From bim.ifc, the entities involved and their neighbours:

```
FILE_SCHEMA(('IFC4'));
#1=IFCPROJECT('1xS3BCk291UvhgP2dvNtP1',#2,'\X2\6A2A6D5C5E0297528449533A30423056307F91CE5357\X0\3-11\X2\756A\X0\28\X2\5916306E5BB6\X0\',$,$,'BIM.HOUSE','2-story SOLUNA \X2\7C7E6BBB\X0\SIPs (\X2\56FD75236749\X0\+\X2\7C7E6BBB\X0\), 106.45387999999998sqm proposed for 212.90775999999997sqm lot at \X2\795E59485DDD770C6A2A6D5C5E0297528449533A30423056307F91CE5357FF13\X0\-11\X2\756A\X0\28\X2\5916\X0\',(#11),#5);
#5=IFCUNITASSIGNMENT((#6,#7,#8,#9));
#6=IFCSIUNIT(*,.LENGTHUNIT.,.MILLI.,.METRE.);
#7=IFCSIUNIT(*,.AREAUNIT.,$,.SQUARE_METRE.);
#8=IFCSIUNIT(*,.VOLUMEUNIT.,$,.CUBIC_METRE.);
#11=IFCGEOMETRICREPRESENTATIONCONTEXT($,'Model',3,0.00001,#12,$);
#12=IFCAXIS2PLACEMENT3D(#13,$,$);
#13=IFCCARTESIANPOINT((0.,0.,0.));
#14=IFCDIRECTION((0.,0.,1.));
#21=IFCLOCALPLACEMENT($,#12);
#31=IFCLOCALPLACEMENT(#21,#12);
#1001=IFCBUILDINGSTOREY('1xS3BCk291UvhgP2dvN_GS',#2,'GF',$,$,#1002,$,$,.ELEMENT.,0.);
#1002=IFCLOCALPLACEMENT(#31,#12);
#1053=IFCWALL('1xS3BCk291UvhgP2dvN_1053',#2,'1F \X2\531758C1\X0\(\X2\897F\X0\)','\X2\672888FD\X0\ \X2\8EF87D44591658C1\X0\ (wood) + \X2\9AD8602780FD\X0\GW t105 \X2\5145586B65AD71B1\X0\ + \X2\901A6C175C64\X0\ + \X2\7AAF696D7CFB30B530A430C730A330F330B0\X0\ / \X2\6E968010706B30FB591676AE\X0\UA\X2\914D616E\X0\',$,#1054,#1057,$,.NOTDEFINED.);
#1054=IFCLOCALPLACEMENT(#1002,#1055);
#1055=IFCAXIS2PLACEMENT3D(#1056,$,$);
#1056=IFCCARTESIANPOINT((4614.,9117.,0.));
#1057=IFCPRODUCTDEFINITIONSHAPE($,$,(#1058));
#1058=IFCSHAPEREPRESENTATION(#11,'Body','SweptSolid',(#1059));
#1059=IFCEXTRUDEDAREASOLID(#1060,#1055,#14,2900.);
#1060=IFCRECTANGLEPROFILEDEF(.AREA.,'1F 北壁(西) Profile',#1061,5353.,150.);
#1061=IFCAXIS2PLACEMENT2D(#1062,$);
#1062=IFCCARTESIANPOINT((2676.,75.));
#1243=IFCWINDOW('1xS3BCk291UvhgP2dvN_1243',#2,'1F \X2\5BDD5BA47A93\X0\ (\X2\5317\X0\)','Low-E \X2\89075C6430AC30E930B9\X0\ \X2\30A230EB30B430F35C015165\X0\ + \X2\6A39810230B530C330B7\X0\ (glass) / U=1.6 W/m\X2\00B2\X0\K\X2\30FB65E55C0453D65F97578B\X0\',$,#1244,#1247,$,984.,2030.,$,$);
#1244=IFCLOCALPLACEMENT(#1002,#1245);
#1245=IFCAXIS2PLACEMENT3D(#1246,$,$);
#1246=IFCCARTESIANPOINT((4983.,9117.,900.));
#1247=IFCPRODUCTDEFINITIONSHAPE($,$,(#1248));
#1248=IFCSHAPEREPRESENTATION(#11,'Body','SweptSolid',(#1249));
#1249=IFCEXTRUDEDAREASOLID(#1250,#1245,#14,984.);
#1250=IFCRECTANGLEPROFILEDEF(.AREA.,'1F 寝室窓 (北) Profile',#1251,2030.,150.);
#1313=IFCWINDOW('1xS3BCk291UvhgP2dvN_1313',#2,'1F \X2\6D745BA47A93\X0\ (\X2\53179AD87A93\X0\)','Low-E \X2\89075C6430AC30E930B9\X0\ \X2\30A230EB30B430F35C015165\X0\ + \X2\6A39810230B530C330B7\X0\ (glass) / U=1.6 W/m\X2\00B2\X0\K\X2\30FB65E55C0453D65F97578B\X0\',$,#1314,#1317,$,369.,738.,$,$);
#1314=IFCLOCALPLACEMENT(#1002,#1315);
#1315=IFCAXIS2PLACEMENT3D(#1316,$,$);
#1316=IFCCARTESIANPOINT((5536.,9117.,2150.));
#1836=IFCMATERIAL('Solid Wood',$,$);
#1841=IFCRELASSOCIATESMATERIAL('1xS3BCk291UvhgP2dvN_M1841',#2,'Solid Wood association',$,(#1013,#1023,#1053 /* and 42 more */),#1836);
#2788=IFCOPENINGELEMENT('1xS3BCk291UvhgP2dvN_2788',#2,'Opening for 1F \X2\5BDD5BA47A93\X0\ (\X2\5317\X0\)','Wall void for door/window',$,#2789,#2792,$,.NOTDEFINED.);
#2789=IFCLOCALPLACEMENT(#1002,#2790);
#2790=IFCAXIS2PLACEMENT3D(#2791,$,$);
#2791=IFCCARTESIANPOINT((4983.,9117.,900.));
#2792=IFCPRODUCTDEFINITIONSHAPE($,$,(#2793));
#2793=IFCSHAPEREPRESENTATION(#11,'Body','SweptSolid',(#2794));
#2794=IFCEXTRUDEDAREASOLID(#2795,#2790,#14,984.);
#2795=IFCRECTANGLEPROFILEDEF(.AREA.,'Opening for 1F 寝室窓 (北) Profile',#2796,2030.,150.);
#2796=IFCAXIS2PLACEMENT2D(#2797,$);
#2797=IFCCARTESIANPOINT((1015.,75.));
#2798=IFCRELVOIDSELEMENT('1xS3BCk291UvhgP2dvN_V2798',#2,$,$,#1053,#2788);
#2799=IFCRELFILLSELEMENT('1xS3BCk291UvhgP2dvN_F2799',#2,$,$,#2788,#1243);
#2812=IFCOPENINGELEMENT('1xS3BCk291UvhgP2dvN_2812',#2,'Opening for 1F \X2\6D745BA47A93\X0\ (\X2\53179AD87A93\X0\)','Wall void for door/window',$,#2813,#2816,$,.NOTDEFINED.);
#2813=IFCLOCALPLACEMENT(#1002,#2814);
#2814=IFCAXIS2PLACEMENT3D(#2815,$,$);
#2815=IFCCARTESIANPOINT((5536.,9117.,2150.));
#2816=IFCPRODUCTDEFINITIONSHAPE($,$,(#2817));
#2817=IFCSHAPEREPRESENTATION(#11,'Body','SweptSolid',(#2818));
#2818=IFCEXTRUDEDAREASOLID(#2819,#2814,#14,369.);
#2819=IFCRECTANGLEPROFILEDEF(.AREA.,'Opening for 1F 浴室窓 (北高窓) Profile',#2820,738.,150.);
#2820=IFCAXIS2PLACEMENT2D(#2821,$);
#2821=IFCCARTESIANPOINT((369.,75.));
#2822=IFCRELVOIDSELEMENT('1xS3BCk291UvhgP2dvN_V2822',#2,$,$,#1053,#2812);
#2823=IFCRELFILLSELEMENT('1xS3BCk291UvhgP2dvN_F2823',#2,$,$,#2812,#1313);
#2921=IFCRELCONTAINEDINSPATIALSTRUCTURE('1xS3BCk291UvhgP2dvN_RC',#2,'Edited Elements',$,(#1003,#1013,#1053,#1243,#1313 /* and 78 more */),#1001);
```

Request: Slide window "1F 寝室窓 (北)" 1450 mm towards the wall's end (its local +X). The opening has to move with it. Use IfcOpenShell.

```python
import ifcopenshell
import ifcopenshell.api.geometry
import ifcopenshell.util.placement
import ifcopenshell.util.unit

model = ifcopenshell.open("bim.ifc")
unit_scale = ifcopenshell.util.unit.calculate_unit_scale(model)

window = model.by_id(1243)
opening = window.FillsVoids[0].RelatingOpeningElement
wall = opening.VoidsElements[0].RelatingBuildingElement

wall_matrix = ifcopenshell.util.placement.get_local_placement(wall.ObjectPlacement)
shift = wall_matrix[:3, 0] * 1.45 / unit_scale
before = ifcopenshell.util.placement.get_local_placement(window.ObjectPlacement)[:3, 3].copy()

# The window is not placed relative to its opening, so move both.
for product in (opening, window):
    matrix = ifcopenshell.util.placement.get_local_placement(product.ObjectPlacement)
    matrix[:3, 3] += shift
    ifcopenshell.api.geometry.edit_object_placement(model, product=product, matrix=matrix, is_si=False)

after = ifcopenshell.util.placement.get_local_placement(window.ObjectPlacement)[:3, 3]
print("window moved by", (after - before).round(3) + 0.0)

model.write("bim_v2.ifc")
```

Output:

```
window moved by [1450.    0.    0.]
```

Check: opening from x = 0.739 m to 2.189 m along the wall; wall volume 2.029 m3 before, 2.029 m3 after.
